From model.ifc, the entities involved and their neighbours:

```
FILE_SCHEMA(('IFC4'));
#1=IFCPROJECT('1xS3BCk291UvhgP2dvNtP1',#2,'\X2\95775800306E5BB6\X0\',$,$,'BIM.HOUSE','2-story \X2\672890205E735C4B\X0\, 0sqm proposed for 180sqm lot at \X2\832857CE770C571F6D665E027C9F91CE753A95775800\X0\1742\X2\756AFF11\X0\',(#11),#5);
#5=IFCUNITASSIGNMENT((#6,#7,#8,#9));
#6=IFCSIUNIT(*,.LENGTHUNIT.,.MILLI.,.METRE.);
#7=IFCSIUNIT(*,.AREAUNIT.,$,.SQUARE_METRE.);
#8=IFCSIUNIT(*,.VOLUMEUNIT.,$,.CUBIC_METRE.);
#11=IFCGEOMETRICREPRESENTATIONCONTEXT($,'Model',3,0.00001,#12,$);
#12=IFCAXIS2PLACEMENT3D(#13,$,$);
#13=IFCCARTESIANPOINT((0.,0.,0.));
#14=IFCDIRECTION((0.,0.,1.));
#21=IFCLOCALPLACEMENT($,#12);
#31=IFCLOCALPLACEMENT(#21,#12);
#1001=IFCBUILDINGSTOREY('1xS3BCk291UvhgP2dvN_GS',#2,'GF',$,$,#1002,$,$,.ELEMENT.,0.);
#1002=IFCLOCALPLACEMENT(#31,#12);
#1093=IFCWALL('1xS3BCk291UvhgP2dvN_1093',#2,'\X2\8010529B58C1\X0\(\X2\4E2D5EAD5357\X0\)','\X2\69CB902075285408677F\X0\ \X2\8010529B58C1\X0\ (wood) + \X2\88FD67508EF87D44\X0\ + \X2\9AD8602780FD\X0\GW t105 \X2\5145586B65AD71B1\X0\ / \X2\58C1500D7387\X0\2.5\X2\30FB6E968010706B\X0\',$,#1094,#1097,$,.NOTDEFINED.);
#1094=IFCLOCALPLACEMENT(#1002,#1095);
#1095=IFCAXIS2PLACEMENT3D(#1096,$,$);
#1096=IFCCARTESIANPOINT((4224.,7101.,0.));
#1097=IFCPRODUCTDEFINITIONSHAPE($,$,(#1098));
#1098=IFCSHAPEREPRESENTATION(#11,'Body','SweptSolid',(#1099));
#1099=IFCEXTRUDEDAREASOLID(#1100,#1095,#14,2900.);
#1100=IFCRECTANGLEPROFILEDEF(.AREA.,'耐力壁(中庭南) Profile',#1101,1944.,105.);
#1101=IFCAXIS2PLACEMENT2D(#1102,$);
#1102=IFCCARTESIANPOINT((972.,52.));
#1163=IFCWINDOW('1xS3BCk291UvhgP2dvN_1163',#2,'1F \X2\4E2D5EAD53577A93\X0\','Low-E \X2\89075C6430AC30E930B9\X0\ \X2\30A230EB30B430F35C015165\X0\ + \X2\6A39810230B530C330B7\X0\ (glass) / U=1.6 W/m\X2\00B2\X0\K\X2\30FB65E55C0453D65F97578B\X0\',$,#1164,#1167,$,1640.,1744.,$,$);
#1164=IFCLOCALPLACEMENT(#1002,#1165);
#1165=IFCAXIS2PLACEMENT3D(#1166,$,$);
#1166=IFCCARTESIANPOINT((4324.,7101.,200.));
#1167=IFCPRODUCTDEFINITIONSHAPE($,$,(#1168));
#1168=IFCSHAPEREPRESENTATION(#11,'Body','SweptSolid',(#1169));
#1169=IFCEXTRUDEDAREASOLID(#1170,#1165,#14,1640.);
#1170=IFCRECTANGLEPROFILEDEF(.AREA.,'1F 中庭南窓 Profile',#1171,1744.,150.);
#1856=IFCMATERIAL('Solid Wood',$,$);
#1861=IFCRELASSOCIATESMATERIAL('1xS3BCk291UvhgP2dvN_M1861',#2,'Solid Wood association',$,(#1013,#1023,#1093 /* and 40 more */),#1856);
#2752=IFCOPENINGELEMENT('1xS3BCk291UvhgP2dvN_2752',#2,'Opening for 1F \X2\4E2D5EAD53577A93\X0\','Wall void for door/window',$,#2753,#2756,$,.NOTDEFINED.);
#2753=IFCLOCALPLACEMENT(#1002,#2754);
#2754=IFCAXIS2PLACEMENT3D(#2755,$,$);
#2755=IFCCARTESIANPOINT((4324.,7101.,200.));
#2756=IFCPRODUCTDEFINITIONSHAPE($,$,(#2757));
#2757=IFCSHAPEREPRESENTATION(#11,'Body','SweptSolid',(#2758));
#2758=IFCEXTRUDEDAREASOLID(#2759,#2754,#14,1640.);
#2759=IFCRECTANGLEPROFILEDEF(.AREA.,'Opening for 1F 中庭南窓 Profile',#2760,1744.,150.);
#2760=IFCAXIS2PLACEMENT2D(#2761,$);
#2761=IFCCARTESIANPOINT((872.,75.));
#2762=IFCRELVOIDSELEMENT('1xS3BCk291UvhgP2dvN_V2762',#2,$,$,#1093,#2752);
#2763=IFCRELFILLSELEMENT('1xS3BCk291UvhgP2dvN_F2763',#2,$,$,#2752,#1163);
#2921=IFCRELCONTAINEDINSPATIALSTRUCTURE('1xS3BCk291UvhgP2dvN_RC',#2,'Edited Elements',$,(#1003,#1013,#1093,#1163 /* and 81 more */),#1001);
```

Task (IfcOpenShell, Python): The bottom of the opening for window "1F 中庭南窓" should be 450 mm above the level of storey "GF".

```python
import numpy as np
import ifcopenshell
import ifcopenshell.api.geometry
import ifcopenshell.geom
import ifcopenshell.util.element
import ifcopenshell.util.placement
import ifcopenshell.util.shape
import ifcopenshell.util.unit

model = ifcopenshell.open("model.ifc")
unit_scale = ifcopenshell.util.unit.calculate_unit_scale(model)

window = model.by_guid("1xS3BCk291UvhgP2dvN_1163")
opening = window.FillsVoids[0].RelatingOpeningElement
storey = ifcopenshell.util.element.get_container(window, ifc_class="IfcBuildingStorey")
level = ifcopenshell.util.placement.get_local_placement(storey.ObjectPlacement)[2, 3]

# The opening's origin need not be at the sill, so measure its lowest point.
shape = ifcopenshell.geom.create_shape(ifcopenshell.geom.settings(), opening)
bottom = ifcopenshell.util.shape.get_shape_bottom_elevation(shape, shape.geometry) / unit_scale
dz = level + 450.0 - bottom

shift = np.array([0.0, 0.0, dz])
# The window is not placed relative to its opening, so move both.
for product in (opening, window):
    matrix = ifcopenshell.util.placement.get_local_placement(product.ObjectPlacement)
    matrix[:3, 3] += shift
    ifcopenshell.api.geometry.edit_object_placement(model, product=product, matrix=matrix, is_si=False)

print(f"moved by {dz * unit_scale:+.3f} m")

model.write("model_updated.ifc")
```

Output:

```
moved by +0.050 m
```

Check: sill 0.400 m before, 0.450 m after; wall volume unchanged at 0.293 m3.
